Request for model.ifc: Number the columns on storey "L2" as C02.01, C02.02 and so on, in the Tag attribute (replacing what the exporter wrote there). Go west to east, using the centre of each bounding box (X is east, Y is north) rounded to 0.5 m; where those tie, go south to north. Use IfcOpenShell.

First a look at what the model holds.

```python
import ifcopenshell
import ifcopenshell.util.element
import ifcopenshell.util.placement

model = ifcopenshell.open("model.ifc")
print(model.schema)
storey = next(s for s in model.by_type("IfcBuildingStorey") if s.Name == "L2")
columns = [e for e in ifcopenshell.util.element.get_decomposition(storey) if e.is_a("IfcColumn")]
for e in sorted(columns, key=lambda e: e.id()):
    origin = ifcopenshell.util.placement.get_local_placement(e.ObjectPlacement)[:3, 3]
    print(e.id(), e.Tag, e.Name, origin.round(2) + 0.0, sep=" | ")
```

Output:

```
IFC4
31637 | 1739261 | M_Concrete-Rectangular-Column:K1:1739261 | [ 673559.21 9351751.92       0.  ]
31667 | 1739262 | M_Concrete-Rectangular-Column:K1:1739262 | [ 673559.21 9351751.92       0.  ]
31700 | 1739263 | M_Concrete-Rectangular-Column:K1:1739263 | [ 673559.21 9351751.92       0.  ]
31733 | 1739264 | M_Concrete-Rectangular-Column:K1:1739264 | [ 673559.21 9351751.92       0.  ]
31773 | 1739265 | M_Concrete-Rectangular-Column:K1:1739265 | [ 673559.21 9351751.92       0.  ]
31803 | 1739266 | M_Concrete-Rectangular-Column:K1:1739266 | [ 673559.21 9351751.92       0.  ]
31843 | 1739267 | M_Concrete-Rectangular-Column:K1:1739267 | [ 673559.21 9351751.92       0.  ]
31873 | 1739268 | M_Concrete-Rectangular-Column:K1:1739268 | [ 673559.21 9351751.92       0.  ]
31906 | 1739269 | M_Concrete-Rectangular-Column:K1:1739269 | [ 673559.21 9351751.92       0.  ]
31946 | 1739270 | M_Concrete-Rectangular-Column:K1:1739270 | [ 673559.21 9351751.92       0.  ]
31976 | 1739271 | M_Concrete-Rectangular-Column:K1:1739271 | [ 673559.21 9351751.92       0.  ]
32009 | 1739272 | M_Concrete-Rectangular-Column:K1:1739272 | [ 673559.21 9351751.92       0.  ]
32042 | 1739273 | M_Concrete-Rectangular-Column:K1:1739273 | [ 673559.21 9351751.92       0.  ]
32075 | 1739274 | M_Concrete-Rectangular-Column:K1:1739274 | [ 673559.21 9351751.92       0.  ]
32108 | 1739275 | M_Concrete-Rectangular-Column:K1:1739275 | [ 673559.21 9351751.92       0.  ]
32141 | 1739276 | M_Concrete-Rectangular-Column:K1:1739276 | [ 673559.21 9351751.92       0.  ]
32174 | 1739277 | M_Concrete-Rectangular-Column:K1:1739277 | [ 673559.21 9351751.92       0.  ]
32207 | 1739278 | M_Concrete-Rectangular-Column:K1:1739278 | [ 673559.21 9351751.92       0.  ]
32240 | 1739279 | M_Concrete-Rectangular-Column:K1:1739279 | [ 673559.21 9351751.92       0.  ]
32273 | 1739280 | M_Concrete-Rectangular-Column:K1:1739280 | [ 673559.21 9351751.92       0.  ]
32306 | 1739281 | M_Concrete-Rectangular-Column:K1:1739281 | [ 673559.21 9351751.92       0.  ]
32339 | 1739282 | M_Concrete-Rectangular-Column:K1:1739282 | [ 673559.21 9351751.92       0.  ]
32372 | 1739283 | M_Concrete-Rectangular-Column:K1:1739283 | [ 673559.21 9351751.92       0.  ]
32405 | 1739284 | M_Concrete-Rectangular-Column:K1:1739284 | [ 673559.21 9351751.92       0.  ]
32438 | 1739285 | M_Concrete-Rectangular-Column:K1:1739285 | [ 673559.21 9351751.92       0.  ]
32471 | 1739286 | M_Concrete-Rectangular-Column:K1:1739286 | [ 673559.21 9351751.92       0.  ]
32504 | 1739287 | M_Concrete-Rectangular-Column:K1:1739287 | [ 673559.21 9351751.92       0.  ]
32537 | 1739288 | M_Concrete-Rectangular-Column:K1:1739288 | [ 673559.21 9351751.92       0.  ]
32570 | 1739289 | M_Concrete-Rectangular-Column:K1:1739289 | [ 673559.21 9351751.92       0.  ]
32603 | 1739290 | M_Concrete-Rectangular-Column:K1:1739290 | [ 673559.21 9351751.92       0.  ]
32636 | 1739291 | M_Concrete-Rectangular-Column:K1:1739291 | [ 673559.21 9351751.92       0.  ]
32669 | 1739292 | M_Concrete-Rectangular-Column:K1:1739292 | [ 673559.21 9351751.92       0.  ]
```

```python
import ifcopenshell
import ifcopenshell.geom
import ifcopenshell.util.element
import ifcopenshell.util.shape

model = ifcopenshell.open("model.ifc")
settings = ifcopenshell.geom.settings()
settings.set("use-world-coords", True)


def centre(element):
    shape = ifcopenshell.geom.create_shape(settings, element)
    return ifcopenshell.util.shape.get_bbox_centroid(shape.geometry)


storey = next(s for s in model.by_type("IfcBuildingStorey") if s.Name == "L2")
columns = [e for e in ifcopenshell.util.element.get_decomposition(storey) if e.is_a("IfcColumn")]

# Insertion points can sit at a corner or the storey origin, so sort by the geometry (in metres).
centres = {e: centre(e) for e in columns}
columns.sort(key=lambda e: (round(centres[e][0] / 0.5), centres[e][1]))

for i, e in enumerate(columns, start=1):
    number = f"C02.{i:02d}"
    e.Tag = number
    print(e.id(), number)

model.write("model_rev.ifc")
```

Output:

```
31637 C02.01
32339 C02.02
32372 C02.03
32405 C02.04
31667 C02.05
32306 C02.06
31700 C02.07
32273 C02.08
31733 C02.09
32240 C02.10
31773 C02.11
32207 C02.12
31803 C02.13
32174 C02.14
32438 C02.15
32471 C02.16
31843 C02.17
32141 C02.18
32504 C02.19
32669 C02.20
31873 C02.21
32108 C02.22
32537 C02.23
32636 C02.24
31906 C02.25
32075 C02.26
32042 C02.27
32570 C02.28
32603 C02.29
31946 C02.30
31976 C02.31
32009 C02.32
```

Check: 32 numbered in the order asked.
